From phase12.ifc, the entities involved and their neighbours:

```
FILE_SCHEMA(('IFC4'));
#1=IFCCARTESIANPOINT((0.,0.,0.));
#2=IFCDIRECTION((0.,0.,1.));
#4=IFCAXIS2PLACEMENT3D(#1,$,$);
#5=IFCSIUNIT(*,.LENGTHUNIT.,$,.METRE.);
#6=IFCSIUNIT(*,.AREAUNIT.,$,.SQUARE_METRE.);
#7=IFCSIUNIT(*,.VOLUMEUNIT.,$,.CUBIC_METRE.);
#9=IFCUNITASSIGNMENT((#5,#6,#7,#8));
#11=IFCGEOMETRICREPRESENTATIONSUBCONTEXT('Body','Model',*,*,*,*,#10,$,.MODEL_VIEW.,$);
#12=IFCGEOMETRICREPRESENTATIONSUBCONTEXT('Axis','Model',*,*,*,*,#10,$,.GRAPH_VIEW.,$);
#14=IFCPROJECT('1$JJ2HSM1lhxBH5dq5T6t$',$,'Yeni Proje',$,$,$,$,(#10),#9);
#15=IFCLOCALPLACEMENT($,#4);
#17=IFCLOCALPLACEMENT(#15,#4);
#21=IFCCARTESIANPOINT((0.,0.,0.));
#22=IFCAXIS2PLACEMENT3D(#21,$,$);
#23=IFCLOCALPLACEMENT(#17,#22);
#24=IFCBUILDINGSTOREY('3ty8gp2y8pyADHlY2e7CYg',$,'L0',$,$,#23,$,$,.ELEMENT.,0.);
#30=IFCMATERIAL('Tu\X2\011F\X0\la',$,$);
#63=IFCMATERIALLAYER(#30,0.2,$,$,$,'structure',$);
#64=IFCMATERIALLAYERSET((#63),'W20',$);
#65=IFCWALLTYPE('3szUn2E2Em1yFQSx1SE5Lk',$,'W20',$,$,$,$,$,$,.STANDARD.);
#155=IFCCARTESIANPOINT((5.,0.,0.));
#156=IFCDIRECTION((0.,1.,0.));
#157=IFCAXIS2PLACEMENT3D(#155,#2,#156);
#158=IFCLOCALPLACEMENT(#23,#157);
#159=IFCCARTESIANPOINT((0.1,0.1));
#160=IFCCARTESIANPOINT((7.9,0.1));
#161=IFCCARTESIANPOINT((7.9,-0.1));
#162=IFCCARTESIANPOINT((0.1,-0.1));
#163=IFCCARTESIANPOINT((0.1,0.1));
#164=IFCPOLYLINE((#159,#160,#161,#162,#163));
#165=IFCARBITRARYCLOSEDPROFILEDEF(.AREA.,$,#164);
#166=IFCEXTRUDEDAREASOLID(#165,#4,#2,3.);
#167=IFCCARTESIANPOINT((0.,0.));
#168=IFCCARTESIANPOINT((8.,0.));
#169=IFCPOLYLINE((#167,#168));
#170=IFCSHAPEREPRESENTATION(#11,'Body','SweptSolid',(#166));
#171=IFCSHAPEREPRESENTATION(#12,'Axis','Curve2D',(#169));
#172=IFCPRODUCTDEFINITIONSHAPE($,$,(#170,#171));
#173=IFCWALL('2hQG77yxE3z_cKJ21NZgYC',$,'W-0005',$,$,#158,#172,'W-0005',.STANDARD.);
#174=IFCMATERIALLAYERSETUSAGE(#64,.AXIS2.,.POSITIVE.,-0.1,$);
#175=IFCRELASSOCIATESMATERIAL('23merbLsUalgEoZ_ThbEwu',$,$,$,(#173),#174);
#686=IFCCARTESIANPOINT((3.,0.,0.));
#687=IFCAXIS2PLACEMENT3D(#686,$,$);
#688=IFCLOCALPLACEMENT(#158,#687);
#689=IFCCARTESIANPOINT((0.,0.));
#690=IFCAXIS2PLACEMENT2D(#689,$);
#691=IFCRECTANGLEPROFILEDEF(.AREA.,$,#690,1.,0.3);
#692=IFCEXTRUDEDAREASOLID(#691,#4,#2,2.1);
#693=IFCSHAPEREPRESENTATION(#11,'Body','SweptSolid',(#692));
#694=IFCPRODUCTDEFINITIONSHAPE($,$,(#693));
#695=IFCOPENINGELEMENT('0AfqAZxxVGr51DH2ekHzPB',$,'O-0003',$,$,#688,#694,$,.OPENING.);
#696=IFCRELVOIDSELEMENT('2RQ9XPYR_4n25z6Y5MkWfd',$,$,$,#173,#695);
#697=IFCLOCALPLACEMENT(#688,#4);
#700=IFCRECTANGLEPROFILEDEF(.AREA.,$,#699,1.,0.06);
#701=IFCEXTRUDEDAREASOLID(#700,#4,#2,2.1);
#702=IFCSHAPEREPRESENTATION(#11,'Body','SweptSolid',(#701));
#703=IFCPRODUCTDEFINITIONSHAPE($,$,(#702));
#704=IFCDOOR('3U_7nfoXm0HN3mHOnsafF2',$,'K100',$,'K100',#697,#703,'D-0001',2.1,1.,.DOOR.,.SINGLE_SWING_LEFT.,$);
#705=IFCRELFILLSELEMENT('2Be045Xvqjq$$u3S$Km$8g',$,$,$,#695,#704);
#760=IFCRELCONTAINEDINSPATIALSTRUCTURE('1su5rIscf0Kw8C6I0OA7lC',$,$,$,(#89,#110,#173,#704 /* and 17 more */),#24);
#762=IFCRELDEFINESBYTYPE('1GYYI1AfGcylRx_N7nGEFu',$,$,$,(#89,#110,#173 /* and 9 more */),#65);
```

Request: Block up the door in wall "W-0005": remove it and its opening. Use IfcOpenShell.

```python
import ifcopenshell
import ifcopenshell.api.feature
import ifcopenshell.api.root
import ifcopenshell.geom
import ifcopenshell.util.shape

model = ifcopenshell.open("phase12.ifc")
settings = ifcopenshell.geom.settings()


def volume(element):
    """Net volume in cubic metres, openings subtracted."""
    shape = ifcopenshell.geom.create_shape(settings, element)
    return ifcopenshell.util.shape.get_volume(shape.geometry)


door = model.by_guid("3U_7nfoXm0HN3mHOnsafF2")
opening = door.FillsVoids[0].RelatingOpeningElement
wall = opening.VoidsElements[0].RelatingBuildingElement
before = volume(wall)

ifcopenshell.api.root.remove_product(model, product=door)
ifcopenshell.api.feature.remove_feature(model, feature=opening)

after = volume(wall)

print(f"wall volume {before:.3f} -> {after:.3f} m3")

model.write("phase12_updated.ifc")
```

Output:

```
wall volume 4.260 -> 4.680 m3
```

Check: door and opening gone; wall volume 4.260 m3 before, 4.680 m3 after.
